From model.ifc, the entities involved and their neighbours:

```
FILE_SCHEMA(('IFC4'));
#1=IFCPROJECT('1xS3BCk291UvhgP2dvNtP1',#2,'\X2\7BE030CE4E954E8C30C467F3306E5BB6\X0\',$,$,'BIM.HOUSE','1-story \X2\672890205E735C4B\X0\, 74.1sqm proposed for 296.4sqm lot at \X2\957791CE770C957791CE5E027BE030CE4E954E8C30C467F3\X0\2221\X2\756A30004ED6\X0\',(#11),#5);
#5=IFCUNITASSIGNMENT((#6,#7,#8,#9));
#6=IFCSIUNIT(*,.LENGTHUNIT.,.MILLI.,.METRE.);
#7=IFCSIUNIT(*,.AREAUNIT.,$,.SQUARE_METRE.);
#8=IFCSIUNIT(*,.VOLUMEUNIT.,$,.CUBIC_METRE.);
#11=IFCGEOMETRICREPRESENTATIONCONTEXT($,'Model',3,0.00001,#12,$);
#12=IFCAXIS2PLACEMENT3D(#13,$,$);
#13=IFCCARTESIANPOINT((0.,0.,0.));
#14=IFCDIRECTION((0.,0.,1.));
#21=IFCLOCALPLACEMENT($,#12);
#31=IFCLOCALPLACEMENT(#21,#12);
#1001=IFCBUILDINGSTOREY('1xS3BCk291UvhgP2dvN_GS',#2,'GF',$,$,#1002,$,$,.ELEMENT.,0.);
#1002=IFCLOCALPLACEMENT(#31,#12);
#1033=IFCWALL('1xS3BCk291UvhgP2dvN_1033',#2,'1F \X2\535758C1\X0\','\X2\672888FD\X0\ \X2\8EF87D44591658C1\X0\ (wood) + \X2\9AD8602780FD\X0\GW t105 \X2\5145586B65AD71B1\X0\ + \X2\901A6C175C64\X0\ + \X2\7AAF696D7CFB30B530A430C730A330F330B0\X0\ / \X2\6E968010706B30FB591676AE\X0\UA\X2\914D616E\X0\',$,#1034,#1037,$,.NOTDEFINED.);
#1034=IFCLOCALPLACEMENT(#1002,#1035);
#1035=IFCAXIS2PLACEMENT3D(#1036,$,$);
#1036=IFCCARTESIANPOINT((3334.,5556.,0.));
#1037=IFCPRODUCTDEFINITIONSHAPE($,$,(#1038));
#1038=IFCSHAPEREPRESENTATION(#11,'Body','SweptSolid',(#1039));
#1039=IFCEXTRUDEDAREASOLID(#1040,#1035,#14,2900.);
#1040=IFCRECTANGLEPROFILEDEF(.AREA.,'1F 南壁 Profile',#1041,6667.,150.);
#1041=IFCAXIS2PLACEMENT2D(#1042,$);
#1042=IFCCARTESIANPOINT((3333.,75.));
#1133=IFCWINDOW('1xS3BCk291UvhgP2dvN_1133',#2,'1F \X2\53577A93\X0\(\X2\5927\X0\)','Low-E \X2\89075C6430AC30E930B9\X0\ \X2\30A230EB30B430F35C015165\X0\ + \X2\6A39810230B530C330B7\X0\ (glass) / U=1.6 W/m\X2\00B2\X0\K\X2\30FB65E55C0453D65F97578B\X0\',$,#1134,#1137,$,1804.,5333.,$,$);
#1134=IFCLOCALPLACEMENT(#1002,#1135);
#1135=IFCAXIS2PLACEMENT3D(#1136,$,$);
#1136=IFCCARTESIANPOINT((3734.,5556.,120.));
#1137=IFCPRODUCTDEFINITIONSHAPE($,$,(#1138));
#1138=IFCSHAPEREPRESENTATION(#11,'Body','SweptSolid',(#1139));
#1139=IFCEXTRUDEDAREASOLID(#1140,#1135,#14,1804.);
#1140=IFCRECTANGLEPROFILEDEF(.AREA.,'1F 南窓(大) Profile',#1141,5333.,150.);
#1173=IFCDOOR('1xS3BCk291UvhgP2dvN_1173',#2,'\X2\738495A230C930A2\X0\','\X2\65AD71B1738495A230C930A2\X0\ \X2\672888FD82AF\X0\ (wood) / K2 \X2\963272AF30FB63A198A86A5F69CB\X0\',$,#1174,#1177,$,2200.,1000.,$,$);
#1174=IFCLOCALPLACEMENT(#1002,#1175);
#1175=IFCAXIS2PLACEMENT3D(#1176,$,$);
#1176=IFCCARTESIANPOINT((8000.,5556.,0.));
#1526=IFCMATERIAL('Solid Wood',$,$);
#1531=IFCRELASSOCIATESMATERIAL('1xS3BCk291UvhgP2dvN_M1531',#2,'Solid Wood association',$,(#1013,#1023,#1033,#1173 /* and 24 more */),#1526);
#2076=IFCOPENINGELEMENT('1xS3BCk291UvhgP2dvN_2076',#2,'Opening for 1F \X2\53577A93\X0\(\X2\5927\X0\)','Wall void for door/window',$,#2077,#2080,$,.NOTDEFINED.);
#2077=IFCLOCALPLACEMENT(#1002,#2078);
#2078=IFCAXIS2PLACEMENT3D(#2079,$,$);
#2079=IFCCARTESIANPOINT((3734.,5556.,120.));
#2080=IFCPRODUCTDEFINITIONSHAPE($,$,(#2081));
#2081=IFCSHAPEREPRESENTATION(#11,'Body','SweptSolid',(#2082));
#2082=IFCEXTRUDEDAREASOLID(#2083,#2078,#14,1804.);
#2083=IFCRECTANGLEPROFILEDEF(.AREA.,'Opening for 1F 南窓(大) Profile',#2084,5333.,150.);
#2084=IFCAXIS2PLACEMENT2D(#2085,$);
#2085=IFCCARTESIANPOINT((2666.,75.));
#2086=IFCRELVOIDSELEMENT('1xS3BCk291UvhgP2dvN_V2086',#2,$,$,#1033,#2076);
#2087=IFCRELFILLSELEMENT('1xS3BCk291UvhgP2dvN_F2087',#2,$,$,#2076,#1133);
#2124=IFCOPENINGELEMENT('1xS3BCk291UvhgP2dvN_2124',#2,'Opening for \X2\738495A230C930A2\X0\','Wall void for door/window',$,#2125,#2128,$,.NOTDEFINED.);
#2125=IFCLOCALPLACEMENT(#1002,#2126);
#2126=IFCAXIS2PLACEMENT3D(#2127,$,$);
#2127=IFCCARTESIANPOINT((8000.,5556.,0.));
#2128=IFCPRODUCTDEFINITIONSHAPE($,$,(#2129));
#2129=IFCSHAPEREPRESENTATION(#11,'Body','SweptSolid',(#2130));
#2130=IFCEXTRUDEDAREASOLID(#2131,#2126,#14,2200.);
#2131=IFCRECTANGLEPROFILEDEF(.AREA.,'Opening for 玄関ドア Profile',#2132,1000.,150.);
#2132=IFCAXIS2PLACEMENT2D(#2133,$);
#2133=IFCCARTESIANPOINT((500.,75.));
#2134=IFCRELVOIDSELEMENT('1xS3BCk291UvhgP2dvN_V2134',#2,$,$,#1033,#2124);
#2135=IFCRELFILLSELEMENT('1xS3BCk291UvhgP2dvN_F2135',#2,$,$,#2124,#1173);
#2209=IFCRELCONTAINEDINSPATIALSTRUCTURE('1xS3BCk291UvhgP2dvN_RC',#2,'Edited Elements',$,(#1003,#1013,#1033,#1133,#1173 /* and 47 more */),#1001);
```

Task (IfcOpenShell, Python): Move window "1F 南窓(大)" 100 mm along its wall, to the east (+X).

```python
import ifcopenshell
import ifcopenshell.api.geometry
import ifcopenshell.util.placement
import ifcopenshell.util.unit

model = ifcopenshell.open("model.ifc")
unit_scale = ifcopenshell.util.unit.calculate_unit_scale(model)

window = model.by_id(1133)
opening = window.FillsVoids[0].RelatingOpeningElement
wall = opening.VoidsElements[0].RelatingBuildingElement

wall_matrix = ifcopenshell.util.placement.get_local_placement(wall.ObjectPlacement)
shift = wall_matrix[:3, 0] * 0.1 / unit_scale
before = ifcopenshell.util.placement.get_local_placement(window.ObjectPlacement)[:3, 3].copy()

# The window is not placed relative to its opening, so move both.
for product in (opening, window):
    matrix = ifcopenshell.util.placement.get_local_placement(product.ObjectPlacement)
    matrix[:3, 3] += shift
    ifcopenshell.api.geometry.edit_object_placement(model, product=product, matrix=matrix, is_si=False)

after = ifcopenshell.util.placement.get_local_placement(window.ObjectPlacement)[:3, 3]
print("window moved by", (after - before).round(3) + 0.0)

model.write("model_edited.ifc")
```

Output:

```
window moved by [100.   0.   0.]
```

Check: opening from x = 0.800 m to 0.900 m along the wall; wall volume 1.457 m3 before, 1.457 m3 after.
